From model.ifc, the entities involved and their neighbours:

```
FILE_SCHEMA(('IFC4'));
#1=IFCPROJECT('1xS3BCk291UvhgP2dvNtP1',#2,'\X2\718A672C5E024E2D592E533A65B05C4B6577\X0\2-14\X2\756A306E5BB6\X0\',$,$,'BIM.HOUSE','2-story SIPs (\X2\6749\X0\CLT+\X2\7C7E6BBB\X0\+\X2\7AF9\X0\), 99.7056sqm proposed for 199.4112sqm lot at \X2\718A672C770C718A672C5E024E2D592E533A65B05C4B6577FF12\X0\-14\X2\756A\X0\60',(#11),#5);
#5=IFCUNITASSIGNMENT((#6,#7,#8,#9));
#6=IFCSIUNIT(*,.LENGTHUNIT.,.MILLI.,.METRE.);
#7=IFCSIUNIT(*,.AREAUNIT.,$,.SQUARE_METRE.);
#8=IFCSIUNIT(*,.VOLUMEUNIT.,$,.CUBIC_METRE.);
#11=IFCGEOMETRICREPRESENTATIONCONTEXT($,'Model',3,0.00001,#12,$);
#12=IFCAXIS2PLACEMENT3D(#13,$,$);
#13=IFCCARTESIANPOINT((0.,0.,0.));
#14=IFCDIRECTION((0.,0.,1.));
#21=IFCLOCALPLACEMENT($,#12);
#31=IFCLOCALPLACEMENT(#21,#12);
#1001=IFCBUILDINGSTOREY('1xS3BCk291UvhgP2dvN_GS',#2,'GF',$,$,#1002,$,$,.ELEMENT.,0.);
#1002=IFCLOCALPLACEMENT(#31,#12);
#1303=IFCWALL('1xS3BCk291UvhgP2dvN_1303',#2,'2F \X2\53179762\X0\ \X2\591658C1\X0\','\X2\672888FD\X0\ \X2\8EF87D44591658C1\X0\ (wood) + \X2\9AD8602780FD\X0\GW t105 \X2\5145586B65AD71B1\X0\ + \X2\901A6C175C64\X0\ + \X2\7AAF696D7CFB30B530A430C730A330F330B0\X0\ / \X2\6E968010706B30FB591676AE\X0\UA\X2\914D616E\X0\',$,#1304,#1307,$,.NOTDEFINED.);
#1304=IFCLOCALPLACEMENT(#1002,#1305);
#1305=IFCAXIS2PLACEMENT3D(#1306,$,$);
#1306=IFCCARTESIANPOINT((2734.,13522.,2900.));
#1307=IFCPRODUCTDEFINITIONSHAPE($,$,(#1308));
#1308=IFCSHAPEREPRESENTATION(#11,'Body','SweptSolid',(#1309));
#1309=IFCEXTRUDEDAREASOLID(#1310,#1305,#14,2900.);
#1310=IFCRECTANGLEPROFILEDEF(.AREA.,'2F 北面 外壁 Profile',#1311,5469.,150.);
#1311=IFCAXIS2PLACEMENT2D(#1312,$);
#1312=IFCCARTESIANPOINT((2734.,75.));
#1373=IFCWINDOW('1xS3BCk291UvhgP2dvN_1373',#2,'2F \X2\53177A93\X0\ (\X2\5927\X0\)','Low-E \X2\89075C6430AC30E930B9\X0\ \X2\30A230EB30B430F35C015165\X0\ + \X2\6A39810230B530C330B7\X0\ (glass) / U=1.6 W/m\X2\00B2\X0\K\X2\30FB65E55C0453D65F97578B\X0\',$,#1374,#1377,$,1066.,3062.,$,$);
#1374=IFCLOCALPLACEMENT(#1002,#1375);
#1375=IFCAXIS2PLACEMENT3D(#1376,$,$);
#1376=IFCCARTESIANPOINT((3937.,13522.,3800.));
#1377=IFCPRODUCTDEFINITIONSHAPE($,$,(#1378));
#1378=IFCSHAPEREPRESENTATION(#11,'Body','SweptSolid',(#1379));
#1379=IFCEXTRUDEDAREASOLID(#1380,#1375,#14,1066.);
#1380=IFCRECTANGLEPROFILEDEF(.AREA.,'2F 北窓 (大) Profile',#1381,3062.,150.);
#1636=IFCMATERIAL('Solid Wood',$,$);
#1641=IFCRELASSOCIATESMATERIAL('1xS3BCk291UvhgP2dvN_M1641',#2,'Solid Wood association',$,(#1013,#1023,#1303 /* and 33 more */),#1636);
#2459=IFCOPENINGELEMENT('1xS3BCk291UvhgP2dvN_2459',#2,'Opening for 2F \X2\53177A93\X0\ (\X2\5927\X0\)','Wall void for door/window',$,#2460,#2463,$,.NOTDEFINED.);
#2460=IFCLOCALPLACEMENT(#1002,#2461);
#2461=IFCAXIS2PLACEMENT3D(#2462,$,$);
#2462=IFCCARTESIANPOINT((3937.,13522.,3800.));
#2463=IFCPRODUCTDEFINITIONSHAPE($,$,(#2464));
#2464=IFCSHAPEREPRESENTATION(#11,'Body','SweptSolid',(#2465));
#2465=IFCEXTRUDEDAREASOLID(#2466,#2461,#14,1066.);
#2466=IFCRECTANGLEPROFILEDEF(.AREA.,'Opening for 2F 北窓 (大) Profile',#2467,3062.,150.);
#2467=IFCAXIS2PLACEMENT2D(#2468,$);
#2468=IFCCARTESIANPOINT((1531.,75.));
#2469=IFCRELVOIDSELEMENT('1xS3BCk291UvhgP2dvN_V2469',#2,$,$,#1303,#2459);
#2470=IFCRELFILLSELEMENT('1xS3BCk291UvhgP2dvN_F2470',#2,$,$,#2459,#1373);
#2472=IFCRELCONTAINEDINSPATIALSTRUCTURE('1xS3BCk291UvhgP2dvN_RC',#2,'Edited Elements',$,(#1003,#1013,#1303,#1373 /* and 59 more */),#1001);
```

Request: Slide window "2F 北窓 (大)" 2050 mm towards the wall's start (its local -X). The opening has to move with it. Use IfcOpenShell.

```python
import ifcopenshell
import ifcopenshell.api.geometry
import ifcopenshell.util.placement
import ifcopenshell.util.unit

model = ifcopenshell.open("model.ifc")
unit_scale = ifcopenshell.util.unit.calculate_unit_scale(model)

window = model.by_guid("1xS3BCk291UvhgP2dvN_1373")
opening = window.FillsVoids[0].RelatingOpeningElement
wall = opening.VoidsElements[0].RelatingBuildingElement

wall_matrix = ifcopenshell.util.placement.get_local_placement(wall.ObjectPlacement)
shift = wall_matrix[:3, 0] * -2.05 / unit_scale
before = ifcopenshell.util.placement.get_local_placement(window.ObjectPlacement)[:3, 3].copy()

# The window is not placed relative to its opening, so move both.
for product in (opening, window):
    matrix = ifcopenshell.util.placement.get_local_placement(product.ObjectPlacement)
    matrix[:3, 3] += shift
    ifcopenshell.api.geometry.edit_object_placement(model, product=product, matrix=matrix, is_si=False)

after = ifcopenshell.util.placement.get_local_placement(window.ObjectPlacement)[:3, 3]
print("window moved by", (after - before).round(3) + 0.0)

model.write("model_rev.ifc")
```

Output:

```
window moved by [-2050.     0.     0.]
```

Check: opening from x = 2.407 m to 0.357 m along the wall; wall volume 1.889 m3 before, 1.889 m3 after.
